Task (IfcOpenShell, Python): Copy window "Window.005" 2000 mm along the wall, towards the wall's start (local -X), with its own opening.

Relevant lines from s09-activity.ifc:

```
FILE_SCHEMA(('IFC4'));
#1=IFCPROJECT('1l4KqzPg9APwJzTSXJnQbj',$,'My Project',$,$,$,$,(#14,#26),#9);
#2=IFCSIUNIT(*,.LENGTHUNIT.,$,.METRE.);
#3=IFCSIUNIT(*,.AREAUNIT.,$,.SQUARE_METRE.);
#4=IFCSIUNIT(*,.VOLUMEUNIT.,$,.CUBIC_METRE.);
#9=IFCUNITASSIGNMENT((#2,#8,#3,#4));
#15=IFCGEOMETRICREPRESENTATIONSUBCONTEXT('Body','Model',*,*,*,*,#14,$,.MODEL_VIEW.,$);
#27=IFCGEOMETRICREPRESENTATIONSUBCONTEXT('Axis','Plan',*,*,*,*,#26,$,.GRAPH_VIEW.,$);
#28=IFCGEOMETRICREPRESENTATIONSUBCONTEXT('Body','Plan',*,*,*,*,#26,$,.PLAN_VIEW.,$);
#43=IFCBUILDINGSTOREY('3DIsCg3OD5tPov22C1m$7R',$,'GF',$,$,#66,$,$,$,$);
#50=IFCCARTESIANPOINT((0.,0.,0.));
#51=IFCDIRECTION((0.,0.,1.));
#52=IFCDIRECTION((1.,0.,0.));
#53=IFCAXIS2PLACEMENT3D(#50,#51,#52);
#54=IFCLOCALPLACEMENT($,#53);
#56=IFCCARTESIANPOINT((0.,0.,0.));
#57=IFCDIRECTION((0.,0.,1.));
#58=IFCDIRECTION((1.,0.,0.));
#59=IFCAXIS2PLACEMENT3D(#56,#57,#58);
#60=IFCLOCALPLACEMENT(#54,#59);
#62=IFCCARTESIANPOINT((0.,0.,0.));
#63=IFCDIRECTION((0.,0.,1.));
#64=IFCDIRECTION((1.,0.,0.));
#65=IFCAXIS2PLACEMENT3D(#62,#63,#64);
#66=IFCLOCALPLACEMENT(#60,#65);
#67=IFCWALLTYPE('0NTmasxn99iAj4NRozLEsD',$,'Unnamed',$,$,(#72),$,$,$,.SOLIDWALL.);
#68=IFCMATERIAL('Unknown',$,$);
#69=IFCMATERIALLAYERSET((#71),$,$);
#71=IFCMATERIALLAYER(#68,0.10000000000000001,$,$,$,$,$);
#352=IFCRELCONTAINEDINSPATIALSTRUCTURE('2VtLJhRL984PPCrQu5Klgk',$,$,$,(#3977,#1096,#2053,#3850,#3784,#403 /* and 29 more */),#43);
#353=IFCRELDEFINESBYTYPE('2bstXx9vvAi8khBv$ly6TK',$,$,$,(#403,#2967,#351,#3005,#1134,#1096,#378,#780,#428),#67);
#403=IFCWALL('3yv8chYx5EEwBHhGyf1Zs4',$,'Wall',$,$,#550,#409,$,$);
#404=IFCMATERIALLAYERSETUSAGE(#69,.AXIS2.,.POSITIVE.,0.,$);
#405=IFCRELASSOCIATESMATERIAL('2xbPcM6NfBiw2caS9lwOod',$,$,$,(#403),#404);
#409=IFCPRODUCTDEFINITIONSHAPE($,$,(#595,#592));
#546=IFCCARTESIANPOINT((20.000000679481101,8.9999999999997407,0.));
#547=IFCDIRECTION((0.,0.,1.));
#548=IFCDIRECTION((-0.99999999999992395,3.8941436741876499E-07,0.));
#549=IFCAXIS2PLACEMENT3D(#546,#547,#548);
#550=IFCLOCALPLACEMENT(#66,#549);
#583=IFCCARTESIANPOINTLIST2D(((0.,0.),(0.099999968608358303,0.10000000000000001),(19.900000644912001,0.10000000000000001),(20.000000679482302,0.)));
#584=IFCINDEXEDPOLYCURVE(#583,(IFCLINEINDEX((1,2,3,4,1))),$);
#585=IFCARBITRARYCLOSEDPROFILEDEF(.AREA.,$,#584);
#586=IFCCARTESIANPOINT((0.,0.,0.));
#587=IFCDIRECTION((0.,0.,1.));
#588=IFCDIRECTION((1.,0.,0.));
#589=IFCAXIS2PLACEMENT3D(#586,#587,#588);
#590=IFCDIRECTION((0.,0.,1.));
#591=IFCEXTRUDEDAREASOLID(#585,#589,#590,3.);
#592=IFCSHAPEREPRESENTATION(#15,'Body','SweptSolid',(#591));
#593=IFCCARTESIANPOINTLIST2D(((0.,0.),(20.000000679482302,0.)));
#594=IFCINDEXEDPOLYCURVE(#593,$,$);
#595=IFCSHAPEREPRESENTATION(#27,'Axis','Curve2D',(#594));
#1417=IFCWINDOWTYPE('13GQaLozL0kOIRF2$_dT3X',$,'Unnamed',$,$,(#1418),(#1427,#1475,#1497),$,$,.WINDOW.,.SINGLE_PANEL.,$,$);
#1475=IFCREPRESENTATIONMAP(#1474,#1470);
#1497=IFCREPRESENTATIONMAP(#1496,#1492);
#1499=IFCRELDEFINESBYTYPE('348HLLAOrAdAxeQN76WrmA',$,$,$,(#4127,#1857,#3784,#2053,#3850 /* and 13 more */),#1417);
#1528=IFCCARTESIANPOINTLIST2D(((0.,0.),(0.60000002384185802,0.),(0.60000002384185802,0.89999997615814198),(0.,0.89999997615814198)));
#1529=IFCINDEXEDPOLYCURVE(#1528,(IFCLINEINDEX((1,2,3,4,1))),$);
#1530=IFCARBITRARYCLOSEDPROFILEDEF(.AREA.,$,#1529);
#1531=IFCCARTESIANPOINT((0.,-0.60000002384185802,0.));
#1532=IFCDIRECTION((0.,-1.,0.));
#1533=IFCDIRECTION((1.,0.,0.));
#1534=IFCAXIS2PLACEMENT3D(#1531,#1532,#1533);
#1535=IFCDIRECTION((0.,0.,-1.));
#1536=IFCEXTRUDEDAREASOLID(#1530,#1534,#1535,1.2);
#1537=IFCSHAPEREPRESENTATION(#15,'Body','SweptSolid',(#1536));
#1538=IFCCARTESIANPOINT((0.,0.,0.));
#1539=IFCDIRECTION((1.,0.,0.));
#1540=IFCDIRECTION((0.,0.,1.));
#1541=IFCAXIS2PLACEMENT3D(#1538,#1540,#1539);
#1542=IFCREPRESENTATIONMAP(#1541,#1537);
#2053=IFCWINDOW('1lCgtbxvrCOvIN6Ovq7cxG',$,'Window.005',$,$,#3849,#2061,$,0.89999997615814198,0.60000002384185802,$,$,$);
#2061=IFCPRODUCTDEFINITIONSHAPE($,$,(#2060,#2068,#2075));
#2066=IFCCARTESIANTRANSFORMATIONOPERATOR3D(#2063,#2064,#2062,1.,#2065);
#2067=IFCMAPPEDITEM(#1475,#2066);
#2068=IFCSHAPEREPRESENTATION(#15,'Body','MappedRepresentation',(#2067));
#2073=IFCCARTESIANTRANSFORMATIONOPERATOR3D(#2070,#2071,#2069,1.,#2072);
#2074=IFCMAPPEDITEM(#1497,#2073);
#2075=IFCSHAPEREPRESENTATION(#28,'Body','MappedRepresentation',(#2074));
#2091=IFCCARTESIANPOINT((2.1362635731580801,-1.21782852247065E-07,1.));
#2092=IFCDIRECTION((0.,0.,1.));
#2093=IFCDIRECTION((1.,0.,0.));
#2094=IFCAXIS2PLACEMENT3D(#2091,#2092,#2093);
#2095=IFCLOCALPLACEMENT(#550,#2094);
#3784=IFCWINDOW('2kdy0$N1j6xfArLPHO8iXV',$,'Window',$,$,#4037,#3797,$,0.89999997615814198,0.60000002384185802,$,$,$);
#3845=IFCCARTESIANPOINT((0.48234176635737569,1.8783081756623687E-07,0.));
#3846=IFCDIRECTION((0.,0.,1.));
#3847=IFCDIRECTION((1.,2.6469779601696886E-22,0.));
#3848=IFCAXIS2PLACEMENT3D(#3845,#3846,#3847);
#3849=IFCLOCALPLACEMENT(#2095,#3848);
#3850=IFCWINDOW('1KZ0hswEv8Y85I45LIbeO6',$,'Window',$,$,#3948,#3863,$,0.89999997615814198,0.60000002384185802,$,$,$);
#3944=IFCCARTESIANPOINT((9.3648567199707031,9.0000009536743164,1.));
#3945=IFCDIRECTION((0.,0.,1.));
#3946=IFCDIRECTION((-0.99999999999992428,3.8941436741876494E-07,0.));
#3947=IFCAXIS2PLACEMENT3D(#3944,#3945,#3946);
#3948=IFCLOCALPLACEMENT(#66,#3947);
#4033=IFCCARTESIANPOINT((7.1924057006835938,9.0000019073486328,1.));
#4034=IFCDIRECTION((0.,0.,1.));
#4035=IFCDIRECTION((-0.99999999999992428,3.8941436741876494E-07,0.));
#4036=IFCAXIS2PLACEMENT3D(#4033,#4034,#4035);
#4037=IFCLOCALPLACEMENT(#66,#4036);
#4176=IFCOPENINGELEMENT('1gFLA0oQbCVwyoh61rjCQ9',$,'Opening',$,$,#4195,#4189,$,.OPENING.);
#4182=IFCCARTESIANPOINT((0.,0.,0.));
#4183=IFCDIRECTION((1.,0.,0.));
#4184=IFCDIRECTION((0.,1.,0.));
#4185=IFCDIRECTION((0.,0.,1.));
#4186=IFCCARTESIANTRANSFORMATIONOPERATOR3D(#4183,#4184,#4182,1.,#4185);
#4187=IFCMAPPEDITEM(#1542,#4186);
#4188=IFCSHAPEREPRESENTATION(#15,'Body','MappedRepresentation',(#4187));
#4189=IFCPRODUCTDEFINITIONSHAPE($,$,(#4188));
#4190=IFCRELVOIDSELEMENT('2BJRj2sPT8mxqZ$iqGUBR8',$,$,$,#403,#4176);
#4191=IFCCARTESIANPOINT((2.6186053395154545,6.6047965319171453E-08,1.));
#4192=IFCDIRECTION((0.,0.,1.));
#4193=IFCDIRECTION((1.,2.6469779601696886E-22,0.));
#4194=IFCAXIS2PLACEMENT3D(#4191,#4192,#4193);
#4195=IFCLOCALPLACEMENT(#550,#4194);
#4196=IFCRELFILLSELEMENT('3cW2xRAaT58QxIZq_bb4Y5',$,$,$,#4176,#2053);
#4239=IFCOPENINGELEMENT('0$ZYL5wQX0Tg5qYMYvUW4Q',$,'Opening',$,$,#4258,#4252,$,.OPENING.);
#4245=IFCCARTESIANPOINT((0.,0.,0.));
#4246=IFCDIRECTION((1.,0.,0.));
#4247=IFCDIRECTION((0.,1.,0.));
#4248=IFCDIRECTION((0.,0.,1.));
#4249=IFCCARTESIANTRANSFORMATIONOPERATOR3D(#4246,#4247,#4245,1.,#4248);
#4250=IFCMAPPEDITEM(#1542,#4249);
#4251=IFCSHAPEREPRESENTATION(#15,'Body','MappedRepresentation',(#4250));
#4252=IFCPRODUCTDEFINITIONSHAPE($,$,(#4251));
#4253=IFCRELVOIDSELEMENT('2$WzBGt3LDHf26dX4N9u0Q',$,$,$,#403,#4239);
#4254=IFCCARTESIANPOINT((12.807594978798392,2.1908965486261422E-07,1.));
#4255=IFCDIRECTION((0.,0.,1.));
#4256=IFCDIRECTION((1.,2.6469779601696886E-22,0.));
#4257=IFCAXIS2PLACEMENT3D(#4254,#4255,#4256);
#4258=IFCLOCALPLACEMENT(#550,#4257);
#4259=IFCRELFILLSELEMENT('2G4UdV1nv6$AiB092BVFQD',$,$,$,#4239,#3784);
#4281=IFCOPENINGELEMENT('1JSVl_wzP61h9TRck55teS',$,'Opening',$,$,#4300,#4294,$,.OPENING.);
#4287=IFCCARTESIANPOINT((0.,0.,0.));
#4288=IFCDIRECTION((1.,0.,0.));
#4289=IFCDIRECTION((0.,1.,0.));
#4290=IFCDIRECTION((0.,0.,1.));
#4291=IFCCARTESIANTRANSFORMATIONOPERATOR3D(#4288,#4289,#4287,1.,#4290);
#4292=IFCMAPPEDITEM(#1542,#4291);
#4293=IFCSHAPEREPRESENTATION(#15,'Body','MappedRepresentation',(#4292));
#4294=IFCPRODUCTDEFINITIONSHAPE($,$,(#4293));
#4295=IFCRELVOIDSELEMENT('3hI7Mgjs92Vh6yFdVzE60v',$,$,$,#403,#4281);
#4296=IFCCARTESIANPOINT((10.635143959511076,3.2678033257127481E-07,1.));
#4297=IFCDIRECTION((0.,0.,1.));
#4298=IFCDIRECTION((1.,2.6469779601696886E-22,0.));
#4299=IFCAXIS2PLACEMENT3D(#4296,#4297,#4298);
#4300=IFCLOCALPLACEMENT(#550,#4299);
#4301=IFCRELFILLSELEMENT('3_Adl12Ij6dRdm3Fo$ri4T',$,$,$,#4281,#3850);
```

```python
import ifcopenshell
import ifcopenshell.api.feature
import ifcopenshell.api.geometry
import ifcopenshell.api.root
import ifcopenshell.geom
import ifcopenshell.util.element
import ifcopenshell.util.placement
import ifcopenshell.util.shape
import ifcopenshell.util.unit

model = ifcopenshell.open("s09-activity.ifc")
unit_scale = ifcopenshell.util.unit.calculate_unit_scale(model)
settings = ifcopenshell.geom.settings()


def volume(element):
    """Net volume in cubic metres, openings subtracted."""
    shape = ifcopenshell.geom.create_shape(settings, element)
    return ifcopenshell.util.shape.get_volume(shape.geometry)


window = model.by_guid("1lCgtbxvrCOvIN6Ovq7cxG")
opening = window.FillsVoids[0].RelatingOpeningElement
wall = opening.VoidsElements[0].RelatingBuildingElement
before = volume(wall)
shift = ifcopenshell.util.placement.get_local_placement(wall.ObjectPlacement)[:3, 0] * -2 / unit_scale

# copy_class copies the void relationship, type, container and properties, but no geometry.
new_opening = ifcopenshell.api.root.copy_class(model, product=opening)
new_opening.Representation = ifcopenshell.util.element.copy_deep(
    model, opening.Representation, exclude=["IfcGeometricRepresentationContext", "IfcRepresentationMap"]
)
new_window = ifcopenshell.api.root.copy_class(model, product=window)
new_window.Representation = ifcopenshell.util.element.copy_deep(
    model, window.Representation, exclude=["IfcGeometricRepresentationContext", "IfcRepresentationMap"]
)
ifcopenshell.api.feature.add_filling(model, opening=new_opening, element=new_window)

for old, new in ((opening, new_opening), (window, new_window)):
    matrix = ifcopenshell.util.placement.get_local_placement(old.ObjectPlacement)
    matrix[:3, 3] += shift
    ifcopenshell.api.geometry.edit_object_placement(model, product=new, matrix=matrix, is_si=False)

after = volume(wall)

print(f"wall volume {before:.3f} -> {after:.3f} m3")

model.write("s09-activity-out.ifc")
```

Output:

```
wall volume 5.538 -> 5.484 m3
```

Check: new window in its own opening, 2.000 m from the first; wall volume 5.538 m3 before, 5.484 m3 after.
